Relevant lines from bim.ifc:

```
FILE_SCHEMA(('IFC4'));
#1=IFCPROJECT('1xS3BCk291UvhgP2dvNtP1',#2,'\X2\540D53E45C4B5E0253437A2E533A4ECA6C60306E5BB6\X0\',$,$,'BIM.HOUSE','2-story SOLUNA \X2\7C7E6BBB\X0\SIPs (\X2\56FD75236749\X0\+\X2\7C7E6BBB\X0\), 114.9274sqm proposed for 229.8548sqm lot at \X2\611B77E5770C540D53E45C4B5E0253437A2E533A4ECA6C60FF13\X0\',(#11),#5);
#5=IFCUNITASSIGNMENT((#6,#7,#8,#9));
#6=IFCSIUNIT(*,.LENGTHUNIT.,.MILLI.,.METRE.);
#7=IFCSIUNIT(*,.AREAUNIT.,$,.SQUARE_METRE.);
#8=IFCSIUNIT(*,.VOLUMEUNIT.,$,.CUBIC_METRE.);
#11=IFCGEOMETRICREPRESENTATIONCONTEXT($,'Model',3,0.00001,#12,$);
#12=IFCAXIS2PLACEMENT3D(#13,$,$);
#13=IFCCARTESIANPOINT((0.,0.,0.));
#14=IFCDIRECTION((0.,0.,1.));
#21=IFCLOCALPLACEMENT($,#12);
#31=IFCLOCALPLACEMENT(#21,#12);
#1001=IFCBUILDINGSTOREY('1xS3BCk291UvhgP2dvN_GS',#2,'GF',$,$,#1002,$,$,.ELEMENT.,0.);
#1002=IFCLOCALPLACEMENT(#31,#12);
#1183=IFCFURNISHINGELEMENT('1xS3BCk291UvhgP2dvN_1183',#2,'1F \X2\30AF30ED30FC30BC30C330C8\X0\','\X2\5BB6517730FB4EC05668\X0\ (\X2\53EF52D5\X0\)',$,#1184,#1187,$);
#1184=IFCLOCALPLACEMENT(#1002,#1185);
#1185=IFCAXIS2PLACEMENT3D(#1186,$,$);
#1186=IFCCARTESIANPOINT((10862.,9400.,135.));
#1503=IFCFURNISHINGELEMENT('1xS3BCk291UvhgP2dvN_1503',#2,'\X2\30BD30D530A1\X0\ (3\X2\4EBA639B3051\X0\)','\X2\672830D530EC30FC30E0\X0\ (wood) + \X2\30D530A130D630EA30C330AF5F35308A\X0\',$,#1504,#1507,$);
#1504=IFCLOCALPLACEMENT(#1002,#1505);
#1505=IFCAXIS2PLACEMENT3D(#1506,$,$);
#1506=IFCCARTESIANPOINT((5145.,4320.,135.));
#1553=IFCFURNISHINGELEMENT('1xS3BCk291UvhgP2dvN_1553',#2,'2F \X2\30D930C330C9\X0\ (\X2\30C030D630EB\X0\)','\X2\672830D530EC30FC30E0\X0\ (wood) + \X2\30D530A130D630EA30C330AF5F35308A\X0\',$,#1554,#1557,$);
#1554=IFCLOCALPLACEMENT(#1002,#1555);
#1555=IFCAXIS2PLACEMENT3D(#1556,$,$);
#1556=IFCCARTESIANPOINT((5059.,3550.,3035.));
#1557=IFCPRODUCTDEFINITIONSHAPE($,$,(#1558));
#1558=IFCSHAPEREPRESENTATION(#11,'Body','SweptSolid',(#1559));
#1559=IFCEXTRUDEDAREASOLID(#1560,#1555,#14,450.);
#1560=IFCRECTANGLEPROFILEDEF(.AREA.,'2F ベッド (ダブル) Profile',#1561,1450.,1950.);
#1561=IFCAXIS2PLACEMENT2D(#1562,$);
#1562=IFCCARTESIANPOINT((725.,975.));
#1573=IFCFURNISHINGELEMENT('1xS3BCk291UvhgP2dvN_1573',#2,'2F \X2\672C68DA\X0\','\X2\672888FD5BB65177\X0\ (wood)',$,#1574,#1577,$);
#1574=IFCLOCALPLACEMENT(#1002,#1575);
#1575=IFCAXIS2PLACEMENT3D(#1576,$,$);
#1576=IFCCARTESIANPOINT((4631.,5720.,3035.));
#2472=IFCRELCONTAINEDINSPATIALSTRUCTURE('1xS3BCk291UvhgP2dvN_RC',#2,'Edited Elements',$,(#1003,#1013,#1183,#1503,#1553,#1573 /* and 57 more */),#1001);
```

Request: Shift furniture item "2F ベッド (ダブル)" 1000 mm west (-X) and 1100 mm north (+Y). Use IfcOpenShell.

```python
import ifcopenshell
import ifcopenshell.api.geometry
import ifcopenshell.util.placement
import ifcopenshell.util.unit

model = ifcopenshell.open("bim.ifc")
unit_scale = ifcopenshell.util.unit.calculate_unit_scale(model)

item = model.by_guid("1xS3BCk291UvhgP2dvN_1553")
matrix = ifcopenshell.util.placement.get_local_placement(item.ObjectPlacement)
matrix[0, 3] -= 1 / unit_scale
matrix[1, 3] += 1.1 / unit_scale
ifcopenshell.api.geometry.edit_object_placement(model, product=item, matrix=matrix, is_si=False)

print(ifcopenshell.util.placement.get_local_placement(item.ObjectPlacement).round(3) + 0.0)

model.write("bim_rev.ifc")
```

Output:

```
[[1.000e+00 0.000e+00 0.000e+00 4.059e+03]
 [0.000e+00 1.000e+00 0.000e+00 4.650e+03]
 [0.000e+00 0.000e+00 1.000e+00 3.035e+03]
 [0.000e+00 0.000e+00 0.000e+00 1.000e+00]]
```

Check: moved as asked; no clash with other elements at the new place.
